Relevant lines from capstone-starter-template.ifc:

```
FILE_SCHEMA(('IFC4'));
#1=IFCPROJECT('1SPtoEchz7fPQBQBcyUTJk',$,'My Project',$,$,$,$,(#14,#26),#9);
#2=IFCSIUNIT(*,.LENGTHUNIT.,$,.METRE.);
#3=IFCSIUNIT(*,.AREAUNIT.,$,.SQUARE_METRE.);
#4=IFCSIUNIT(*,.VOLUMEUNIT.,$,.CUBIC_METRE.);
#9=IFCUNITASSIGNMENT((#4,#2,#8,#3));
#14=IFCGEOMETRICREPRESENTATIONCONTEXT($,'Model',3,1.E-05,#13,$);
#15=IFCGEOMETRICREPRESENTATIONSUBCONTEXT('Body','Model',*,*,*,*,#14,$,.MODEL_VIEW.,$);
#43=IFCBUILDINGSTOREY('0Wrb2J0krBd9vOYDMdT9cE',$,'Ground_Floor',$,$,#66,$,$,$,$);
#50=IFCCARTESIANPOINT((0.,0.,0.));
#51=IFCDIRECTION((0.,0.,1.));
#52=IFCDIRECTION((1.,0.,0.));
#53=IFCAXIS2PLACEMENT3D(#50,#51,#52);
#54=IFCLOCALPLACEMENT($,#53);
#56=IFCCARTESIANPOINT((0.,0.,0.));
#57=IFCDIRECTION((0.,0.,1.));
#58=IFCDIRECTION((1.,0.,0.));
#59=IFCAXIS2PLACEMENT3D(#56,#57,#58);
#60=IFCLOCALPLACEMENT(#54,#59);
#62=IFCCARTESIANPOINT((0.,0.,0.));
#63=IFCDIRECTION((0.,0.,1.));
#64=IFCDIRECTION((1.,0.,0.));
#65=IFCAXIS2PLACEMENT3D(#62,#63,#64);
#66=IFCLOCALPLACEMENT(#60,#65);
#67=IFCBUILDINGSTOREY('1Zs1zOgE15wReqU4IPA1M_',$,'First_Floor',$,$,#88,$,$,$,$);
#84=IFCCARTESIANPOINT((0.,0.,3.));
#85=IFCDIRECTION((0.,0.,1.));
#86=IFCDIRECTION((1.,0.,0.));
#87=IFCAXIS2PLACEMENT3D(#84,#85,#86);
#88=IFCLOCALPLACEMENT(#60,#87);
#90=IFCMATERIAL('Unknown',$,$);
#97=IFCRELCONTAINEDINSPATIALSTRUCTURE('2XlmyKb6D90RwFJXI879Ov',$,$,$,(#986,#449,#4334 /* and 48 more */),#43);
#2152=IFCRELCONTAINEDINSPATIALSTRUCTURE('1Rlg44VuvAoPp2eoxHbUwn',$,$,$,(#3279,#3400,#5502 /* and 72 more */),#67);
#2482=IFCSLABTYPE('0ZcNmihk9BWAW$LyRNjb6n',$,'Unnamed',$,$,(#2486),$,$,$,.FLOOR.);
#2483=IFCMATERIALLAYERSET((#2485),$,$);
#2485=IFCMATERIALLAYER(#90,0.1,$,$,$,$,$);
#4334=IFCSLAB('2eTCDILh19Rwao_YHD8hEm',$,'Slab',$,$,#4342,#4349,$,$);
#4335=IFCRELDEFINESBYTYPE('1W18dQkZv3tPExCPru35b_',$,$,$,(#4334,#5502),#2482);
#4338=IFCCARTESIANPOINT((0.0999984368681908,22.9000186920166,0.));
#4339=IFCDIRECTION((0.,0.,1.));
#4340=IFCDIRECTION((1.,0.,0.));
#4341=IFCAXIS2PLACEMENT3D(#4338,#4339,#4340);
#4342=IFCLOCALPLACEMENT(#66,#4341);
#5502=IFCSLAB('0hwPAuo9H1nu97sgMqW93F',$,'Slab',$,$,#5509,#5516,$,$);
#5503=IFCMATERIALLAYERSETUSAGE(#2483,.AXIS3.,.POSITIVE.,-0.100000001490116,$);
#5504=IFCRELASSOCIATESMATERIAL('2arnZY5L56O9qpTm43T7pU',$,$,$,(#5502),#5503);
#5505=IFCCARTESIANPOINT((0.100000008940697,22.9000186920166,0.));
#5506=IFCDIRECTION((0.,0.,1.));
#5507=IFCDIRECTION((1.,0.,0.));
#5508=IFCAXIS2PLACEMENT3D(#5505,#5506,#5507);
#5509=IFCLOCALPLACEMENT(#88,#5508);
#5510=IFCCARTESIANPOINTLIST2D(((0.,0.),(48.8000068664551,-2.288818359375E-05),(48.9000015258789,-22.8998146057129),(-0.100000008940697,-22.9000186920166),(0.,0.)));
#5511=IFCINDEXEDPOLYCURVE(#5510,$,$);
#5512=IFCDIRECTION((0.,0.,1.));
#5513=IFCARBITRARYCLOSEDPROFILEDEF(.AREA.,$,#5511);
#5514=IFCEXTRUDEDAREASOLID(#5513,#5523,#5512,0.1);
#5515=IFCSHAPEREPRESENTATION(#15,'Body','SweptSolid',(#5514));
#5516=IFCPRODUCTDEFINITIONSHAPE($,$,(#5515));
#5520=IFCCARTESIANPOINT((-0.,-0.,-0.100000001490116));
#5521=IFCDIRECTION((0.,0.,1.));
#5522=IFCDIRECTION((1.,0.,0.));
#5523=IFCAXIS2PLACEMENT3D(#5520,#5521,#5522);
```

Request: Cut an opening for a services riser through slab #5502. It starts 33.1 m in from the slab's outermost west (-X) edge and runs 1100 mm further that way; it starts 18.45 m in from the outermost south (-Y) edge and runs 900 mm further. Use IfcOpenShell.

```python
import numpy as np
import ifcopenshell
import ifcopenshell.api.feature
import ifcopenshell.api.geometry
import ifcopenshell.api.root
import ifcopenshell.geom
import ifcopenshell.util.placement
import ifcopenshell.util.representation
import ifcopenshell.util.shape
import ifcopenshell.util.unit

model = ifcopenshell.open("capstone-starter-template.ifc")
unit_scale = ifcopenshell.util.unit.calculate_unit_scale(model)
settings = ifcopenshell.geom.settings()


def volume(element):
    """Net volume in cubic metres, openings subtracted."""
    shape = ifcopenshell.geom.create_shape(settings, element)
    return ifcopenshell.util.shape.get_volume(shape.geometry)


slab = model.by_guid("0hwPAuo9H1nu97sgMqW93F")
before = volume(slab)

# Extent in the slab's own axes, in metres. The edges named are its -X and -Y sides.
slab_shape = ifcopenshell.geom.create_shape(settings, slab)
vertices = ifcopenshell.util.shape.get_vertices(slab_shape.geometry)
x_min, y_min, bottom = vertices.min(axis=0)
top = vertices[:, 2].max()

opening = ifcopenshell.api.root.create_entity(model, ifc_class="IfcOpeningElement", name="Services riser opening", predefined_type="OPENING")
context = ifcopenshell.util.representation.get_context(model, "Model", "Body", "MODEL_VIEW")
width, depth = 1.1, 0.9
outline = [(0.0, 0.0), (width, 0.0), (width, depth), (0.0, depth), (0.0, 0.0)]
# Overshoot both faces by 50 mm so the cut is clean.
shape = ifcopenshell.api.geometry.add_slab_representation(
    model, context=context, depth=top - bottom + 0.1, polyline=outline
)
ifcopenshell.api.geometry.assign_representation(model, product=opening, representation=shape)

matrix = ifcopenshell.util.placement.get_local_placement(slab.ObjectPlacement)
matrix[:, 3] = matrix @ np.append(np.array([x_min + 33.1, y_min + 18.45, bottom - 0.05]) / unit_scale, 1.0)
ifcopenshell.api.geometry.edit_object_placement(model, product=opening, matrix=matrix, is_si=False)
ifcopenshell.api.feature.add_feature(model, feature=opening, element=slab)

after = volume(slab)

print(f"slab volume {before:.3f} -> {after:.3f} m3")

model.write("capstone-starter-template_updated.ifc")
```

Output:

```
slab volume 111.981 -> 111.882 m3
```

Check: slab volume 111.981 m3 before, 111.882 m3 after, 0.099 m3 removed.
